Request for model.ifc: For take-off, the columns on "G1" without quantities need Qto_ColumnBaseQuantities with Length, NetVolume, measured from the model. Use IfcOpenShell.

First a look at what the model holds.

```python
import ifcopenshell
import ifcopenshell.util.element
import ifcopenshell.util.unit

model = ifcopenshell.open("model.ifc")
print(model.schema)
for unit_type in ("LENGTHUNIT", "AREAUNIT", "VOLUMEUNIT"):
    print(unit_type, ifcopenshell.util.unit.calculate_unit_scale(model, unit_type))
storey = next(s for s in model.by_type("IfcBuildingStorey") if s.Name == "G1")
columns = [e for e in ifcopenshell.util.element.get_decomposition(storey) if e.is_a("IfcColumn")]
for e in sorted(columns, key=lambda e: e.id()):
    print(e.id(), e.is_a(), e.Name, list(ifcopenshell.util.element.get_psets(e, qtos_only=True)), sep=" | ")
```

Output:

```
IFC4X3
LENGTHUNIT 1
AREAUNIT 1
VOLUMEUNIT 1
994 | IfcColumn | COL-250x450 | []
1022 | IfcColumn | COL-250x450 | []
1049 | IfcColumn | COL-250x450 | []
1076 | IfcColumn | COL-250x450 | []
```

```python
import ifcopenshell
import ifcopenshell.api.pset
import ifcopenshell.geom
import ifcopenshell.util.element
import ifcopenshell.util.shape
import ifcopenshell.util.unit

model = ifcopenshell.open("model.ifc")
unit_scale = ifcopenshell.util.unit.calculate_unit_scale(model)
volume_scale = ifcopenshell.util.unit.calculate_unit_scale(model, "VOLUMEUNIT")
settings = ifcopenshell.geom.settings()

storey = next(s for s in model.by_type("IfcBuildingStorey") if s.Name == "G1")
columns = [e for e in ifcopenshell.util.element.get_decomposition(storey) if e.is_a("IfcColumn")]

for e in sorted(columns, key=lambda e: e.id()):
    if ifcopenshell.util.element.get_psets(e, qtos_only=True, should_inherit=False):
        continue
    # Geometry comes back in metres, in the element's own axes.
    shape = ifcopenshell.geom.create_shape(settings, e)
    values = {
        "Length": ifcopenshell.util.shape.get_z(shape.geometry) / unit_scale,
        "NetVolume": ifcopenshell.util.shape.get_volume(shape.geometry) / volume_scale,
    }
    qto = ifcopenshell.api.pset.add_qto(model, product=e, name="Qto_ColumnBaseQuantities")
    ifcopenshell.api.pset.edit_qto(model, qto=qto, properties=values)
    print(e.id(), {k: round(v, 3) for k, v in values.items()})

model.write("model_v2.ifc")
```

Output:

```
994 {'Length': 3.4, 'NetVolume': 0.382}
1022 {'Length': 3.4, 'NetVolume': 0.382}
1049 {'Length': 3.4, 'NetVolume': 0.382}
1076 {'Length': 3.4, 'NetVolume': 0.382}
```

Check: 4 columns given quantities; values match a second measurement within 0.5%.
